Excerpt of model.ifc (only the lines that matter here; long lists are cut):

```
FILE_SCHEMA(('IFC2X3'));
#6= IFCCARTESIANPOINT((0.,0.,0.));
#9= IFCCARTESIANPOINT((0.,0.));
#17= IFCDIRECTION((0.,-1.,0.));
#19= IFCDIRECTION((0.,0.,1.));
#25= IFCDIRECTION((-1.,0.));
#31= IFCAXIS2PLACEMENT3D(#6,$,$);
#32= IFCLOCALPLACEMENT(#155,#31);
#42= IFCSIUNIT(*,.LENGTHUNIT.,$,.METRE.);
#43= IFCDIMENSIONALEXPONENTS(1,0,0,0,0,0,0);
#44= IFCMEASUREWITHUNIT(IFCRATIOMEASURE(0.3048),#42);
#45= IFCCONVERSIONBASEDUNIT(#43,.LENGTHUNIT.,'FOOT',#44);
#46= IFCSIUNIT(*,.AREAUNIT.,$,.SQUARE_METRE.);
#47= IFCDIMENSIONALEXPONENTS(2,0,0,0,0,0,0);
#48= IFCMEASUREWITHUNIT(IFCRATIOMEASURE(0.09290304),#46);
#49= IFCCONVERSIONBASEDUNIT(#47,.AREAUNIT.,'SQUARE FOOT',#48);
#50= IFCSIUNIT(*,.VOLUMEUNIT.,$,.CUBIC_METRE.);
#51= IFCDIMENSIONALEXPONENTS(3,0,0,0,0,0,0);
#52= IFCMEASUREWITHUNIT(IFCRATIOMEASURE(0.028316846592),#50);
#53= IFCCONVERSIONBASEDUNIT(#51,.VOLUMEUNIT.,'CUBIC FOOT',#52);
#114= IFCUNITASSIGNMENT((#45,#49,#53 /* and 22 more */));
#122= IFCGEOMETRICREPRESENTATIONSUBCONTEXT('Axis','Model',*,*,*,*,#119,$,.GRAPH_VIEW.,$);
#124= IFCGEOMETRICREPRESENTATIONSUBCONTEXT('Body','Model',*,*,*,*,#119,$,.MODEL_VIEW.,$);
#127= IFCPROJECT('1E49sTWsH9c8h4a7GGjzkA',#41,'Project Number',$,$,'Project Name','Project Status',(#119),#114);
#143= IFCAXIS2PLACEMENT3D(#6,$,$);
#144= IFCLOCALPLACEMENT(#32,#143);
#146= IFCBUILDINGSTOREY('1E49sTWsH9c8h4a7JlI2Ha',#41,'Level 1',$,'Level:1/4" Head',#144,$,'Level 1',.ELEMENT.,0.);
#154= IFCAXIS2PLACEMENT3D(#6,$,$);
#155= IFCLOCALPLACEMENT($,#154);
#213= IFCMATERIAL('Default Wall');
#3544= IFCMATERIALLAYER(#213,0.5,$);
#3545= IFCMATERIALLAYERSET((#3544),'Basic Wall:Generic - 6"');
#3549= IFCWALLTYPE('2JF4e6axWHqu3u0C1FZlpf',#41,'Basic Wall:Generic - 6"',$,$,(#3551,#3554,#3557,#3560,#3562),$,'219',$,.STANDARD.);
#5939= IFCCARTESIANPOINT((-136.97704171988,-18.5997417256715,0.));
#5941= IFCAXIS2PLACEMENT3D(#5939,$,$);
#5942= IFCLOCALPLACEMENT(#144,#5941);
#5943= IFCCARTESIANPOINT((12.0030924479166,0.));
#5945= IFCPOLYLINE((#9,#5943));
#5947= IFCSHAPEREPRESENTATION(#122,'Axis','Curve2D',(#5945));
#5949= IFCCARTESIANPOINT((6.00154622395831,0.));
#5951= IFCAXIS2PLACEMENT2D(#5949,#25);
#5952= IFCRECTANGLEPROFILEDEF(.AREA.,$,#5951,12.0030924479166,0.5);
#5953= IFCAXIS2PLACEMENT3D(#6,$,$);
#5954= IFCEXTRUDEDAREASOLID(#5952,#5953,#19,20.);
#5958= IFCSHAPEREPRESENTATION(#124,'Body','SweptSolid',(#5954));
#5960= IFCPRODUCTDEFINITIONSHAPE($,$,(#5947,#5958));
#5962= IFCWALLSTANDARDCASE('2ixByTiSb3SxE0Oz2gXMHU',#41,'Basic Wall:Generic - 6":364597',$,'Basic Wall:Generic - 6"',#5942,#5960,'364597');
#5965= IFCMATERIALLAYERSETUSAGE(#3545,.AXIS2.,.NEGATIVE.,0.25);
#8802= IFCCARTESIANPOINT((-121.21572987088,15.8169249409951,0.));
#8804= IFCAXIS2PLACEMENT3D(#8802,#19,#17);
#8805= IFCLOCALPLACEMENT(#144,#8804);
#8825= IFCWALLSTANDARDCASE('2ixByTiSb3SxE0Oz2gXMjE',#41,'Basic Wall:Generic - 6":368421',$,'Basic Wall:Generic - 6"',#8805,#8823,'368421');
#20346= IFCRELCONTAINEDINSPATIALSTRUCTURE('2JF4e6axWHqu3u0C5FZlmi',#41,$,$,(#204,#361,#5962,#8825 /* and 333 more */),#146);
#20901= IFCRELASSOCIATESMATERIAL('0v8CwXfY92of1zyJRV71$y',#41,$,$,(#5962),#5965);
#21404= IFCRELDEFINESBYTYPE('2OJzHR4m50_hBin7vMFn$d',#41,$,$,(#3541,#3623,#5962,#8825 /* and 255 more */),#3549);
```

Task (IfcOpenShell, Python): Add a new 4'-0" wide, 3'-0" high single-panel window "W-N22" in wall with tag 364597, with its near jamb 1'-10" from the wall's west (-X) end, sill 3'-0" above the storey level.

```python
import numpy as np
import ifcopenshell
import ifcopenshell.api.feature
import ifcopenshell.api.geometry
import ifcopenshell.api.root
import ifcopenshell.api.spatial
import ifcopenshell.api.type
import ifcopenshell.geom
import ifcopenshell.util.element
import ifcopenshell.util.placement
import ifcopenshell.util.representation
import ifcopenshell.util.shape
import ifcopenshell.util.unit

model = ifcopenshell.open("model.ifc")
unit_scale = ifcopenshell.util.unit.calculate_unit_scale(model)
settings = ifcopenshell.geom.settings()


def volume(element):
    """Net volume in cubic metres, openings subtracted."""
    shape = ifcopenshell.geom.create_shape(settings, element)
    return ifcopenshell.util.shape.get_volume(shape.geometry)


wall = model.by_guid("2ixByTiSb3SxE0Oz2gXMHU")
storey = ifcopenshell.util.element.get_container(wall, ifc_class="IfcBuildingStorey")
context = ifcopenshell.util.representation.get_context(model, "Model", "Body", "MODEL_VIEW")
before = volume(wall)

width, height, from_end, sill = 1.2192, 0.9144, 0.5588, 0.9144  # metres

# The wall runs along its own X axis, and the end named is its -X end.
wall_shape = ifcopenshell.geom.create_shape(settings, wall)
x, y, z = ifcopenshell.util.shape.get_vertices(wall_shape.geometry).T
start = x.min() + from_end
face, thickness = float(y.min()), float(y.max() - y.min())
wall_matrix = ifcopenshell.util.placement.get_local_placement(wall.ObjectPlacement)
level = ifcopenshell.util.placement.get_local_placement(storey.ObjectPlacement)[2, 3]


def in_wall(x, y):
    """Placement at x, y metres in the wall's axes, at sill height."""
    matrix = wall_matrix.copy()
    matrix[:, 3] = wall_matrix @ np.array([x / unit_scale, y / unit_scale, 0.0, 1.0])
    matrix[2, 3] = level + sill / unit_scale
    return matrix


# Opening: a box that overshoots both wall faces by 50 mm.
opening = ifcopenshell.api.root.create_entity(model, ifc_class="IfcOpeningElement")
box = ifcopenshell.api.geometry.add_wall_representation(
    model, context=context, length=width, height=height, thickness=thickness + 0.1
)
ifcopenshell.api.geometry.assign_representation(model, product=opening, representation=box)
ifcopenshell.api.geometry.edit_object_placement(model, product=opening, matrix=in_wall(start, face - 0.05), is_si=False)
ifcopenshell.api.feature.add_feature(model, feature=opening, element=wall)

window = ifcopenshell.api.root.create_entity(model, ifc_class="IfcWindow", name="W-N22")
window.OverallWidth, window.OverallHeight = width / unit_scale, height / unit_scale
body = ifcopenshell.api.geometry.add_window_representation(
    model,
    context=context,
    overall_width=window.OverallWidth,
    overall_height=window.OverallHeight,
    partition_type="SINGLE_PANEL",
)
ifcopenshell.api.geometry.assign_representation(model, product=window, representation=body)
ifcopenshell.api.spatial.assign_container(model, products=[window], relating_structure=storey)
fills = ifcopenshell.api.feature.add_filling(model, opening=opening, element=window)
fills.OwnerHistory = window.OwnerHistory  # required in IFC2X3

# IFC2X3 keeps the operation on the window style.
style = ifcopenshell.api.root.create_entity(model, ifc_class="IfcWindowStyle", name="W-N22")
style.OperationType, style.ConstructionType = "SINGLE_PANEL", "NOTDEFINED"
style.ParameterTakesPrecedence = style.Sizeable = False
ifcopenshell.api.type.assign_type(model, related_objects=[window], relating_type=style)

# Centre the window in the wall's thickness.
ifcopenshell.api.geometry.edit_object_placement(model, product=window, matrix=in_wall(start, face), is_si=False)
window_shape = ifcopenshell.geom.create_shape(settings, window)
depth = ifcopenshell.util.shape.get_vertices(window_shape.geometry)[:, 1]
offset = face + thickness / 2 - (depth.min() + depth.max()) / 2
ifcopenshell.api.geometry.edit_object_placement(model, product=window, matrix=in_wall(start, offset), is_si=False)

after = volume(wall)

print(f"wall volume {before:.3f} -> {after:.3f} m3")

model.write("model_updated.ifc")
```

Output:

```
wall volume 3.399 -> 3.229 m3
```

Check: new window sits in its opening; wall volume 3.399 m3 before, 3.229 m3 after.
